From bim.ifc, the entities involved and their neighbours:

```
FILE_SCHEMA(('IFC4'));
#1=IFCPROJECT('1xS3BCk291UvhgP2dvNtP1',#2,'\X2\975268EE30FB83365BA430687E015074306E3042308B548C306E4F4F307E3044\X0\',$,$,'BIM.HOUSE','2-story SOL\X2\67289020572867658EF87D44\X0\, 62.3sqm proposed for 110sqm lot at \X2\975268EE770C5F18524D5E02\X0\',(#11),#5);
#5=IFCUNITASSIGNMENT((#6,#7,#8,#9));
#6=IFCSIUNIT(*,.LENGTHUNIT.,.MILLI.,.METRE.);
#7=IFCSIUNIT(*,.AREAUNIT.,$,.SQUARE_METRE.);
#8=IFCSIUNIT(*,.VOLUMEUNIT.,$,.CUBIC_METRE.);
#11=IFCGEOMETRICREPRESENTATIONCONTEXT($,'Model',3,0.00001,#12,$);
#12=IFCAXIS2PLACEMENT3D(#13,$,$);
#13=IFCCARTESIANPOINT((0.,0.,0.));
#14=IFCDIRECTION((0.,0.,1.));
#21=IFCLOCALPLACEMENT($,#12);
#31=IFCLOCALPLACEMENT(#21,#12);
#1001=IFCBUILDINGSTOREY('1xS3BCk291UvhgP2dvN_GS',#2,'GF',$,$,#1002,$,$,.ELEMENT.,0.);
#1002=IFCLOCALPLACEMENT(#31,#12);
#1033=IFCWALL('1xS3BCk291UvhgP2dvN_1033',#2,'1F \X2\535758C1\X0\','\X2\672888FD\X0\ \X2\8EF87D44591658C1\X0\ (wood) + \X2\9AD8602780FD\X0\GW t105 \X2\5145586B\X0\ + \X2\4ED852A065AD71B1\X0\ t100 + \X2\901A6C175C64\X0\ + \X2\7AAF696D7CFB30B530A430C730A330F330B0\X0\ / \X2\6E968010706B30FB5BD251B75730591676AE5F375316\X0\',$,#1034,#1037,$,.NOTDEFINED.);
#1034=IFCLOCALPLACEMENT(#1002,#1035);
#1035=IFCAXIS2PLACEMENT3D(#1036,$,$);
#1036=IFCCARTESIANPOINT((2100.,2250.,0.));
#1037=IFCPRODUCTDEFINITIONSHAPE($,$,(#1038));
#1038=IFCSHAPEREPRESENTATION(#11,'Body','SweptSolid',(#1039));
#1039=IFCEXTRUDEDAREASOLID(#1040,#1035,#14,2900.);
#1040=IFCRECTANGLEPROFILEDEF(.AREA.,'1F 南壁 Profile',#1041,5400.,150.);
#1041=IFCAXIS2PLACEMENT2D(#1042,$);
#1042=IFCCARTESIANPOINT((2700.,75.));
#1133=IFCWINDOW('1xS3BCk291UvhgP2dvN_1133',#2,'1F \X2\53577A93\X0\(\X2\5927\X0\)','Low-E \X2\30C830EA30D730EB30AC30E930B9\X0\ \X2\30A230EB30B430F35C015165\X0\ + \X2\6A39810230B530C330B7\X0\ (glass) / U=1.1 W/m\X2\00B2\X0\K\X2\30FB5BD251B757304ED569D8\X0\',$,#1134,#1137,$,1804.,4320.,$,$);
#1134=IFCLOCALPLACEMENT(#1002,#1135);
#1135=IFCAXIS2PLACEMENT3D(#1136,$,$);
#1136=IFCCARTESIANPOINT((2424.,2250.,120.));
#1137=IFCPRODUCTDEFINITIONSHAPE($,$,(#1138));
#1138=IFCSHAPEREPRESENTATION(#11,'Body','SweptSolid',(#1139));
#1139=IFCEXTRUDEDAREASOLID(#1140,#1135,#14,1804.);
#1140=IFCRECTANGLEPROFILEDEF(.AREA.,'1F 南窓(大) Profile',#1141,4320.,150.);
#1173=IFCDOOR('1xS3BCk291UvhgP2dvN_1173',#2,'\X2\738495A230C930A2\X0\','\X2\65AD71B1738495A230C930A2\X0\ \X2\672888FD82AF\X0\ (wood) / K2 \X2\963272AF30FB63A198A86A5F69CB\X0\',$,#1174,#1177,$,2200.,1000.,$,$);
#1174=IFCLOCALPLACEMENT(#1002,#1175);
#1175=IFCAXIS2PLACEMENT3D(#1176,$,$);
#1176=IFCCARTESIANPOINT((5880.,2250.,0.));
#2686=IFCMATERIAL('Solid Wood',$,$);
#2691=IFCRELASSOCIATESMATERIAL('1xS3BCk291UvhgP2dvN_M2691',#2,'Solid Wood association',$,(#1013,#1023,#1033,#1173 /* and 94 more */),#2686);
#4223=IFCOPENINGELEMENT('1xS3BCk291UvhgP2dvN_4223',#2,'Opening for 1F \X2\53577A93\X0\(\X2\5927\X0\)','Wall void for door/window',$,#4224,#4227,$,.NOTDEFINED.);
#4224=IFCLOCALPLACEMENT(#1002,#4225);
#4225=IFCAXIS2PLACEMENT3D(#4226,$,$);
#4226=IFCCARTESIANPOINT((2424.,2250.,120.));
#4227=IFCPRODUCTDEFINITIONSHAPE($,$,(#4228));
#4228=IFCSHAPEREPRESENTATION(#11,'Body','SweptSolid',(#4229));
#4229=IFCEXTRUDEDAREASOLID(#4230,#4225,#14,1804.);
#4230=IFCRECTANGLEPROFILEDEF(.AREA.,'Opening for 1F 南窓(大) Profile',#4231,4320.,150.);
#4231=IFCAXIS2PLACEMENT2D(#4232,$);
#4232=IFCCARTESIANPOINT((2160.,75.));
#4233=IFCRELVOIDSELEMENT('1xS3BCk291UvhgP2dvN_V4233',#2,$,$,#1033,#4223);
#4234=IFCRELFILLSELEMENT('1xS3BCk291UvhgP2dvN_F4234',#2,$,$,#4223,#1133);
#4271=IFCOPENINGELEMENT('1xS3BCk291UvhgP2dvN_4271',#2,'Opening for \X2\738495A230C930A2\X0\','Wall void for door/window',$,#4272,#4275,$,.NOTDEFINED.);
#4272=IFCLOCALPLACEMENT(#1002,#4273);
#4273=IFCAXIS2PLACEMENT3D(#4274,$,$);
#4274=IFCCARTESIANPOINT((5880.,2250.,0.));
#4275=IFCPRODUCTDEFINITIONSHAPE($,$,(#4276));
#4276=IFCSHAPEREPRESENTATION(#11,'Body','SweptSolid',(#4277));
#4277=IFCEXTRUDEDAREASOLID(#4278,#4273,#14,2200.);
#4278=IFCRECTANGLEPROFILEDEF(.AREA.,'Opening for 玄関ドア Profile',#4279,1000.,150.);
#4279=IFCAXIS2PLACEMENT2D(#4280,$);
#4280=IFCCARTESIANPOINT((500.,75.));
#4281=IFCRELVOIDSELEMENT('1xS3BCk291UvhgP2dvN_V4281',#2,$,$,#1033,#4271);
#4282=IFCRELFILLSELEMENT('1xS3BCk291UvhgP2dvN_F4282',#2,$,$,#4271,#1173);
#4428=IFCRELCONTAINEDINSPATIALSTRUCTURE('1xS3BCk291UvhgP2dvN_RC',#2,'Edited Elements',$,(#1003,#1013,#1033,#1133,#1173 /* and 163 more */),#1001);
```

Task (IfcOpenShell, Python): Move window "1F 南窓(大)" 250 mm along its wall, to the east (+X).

```python
import ifcopenshell
import ifcopenshell.api.geometry
import ifcopenshell.util.placement

model = ifcopenshell.open("bim.ifc")

window = model.by_guid("1xS3BCk291UvhgP2dvN_1133")
opening = window.FillsVoids[0].RelatingOpeningElement
wall = opening.VoidsElements[0].RelatingBuildingElement

wall_matrix = ifcopenshell.util.placement.get_local_placement(wall.ObjectPlacement)
shift = wall_matrix[:3, 0] * 250.0
before = ifcopenshell.util.placement.get_local_placement(window.ObjectPlacement)[:3, 3].copy()

# The window is not placed relative to its opening, so move both.
for product in (opening, window):
    matrix = ifcopenshell.util.placement.get_local_placement(product.ObjectPlacement)
    matrix[:3, 3] += shift
    ifcopenshell.api.geometry.edit_object_placement(model, product=product, matrix=matrix, is_si=False)

after = ifcopenshell.util.placement.get_local_placement(window.ObjectPlacement)[:3, 3]
print("window moved by", (after - before).round(3) + 0.0)

model.write("bim_updated.ifc")
```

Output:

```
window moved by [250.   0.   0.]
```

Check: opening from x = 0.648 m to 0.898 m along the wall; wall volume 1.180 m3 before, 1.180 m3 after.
